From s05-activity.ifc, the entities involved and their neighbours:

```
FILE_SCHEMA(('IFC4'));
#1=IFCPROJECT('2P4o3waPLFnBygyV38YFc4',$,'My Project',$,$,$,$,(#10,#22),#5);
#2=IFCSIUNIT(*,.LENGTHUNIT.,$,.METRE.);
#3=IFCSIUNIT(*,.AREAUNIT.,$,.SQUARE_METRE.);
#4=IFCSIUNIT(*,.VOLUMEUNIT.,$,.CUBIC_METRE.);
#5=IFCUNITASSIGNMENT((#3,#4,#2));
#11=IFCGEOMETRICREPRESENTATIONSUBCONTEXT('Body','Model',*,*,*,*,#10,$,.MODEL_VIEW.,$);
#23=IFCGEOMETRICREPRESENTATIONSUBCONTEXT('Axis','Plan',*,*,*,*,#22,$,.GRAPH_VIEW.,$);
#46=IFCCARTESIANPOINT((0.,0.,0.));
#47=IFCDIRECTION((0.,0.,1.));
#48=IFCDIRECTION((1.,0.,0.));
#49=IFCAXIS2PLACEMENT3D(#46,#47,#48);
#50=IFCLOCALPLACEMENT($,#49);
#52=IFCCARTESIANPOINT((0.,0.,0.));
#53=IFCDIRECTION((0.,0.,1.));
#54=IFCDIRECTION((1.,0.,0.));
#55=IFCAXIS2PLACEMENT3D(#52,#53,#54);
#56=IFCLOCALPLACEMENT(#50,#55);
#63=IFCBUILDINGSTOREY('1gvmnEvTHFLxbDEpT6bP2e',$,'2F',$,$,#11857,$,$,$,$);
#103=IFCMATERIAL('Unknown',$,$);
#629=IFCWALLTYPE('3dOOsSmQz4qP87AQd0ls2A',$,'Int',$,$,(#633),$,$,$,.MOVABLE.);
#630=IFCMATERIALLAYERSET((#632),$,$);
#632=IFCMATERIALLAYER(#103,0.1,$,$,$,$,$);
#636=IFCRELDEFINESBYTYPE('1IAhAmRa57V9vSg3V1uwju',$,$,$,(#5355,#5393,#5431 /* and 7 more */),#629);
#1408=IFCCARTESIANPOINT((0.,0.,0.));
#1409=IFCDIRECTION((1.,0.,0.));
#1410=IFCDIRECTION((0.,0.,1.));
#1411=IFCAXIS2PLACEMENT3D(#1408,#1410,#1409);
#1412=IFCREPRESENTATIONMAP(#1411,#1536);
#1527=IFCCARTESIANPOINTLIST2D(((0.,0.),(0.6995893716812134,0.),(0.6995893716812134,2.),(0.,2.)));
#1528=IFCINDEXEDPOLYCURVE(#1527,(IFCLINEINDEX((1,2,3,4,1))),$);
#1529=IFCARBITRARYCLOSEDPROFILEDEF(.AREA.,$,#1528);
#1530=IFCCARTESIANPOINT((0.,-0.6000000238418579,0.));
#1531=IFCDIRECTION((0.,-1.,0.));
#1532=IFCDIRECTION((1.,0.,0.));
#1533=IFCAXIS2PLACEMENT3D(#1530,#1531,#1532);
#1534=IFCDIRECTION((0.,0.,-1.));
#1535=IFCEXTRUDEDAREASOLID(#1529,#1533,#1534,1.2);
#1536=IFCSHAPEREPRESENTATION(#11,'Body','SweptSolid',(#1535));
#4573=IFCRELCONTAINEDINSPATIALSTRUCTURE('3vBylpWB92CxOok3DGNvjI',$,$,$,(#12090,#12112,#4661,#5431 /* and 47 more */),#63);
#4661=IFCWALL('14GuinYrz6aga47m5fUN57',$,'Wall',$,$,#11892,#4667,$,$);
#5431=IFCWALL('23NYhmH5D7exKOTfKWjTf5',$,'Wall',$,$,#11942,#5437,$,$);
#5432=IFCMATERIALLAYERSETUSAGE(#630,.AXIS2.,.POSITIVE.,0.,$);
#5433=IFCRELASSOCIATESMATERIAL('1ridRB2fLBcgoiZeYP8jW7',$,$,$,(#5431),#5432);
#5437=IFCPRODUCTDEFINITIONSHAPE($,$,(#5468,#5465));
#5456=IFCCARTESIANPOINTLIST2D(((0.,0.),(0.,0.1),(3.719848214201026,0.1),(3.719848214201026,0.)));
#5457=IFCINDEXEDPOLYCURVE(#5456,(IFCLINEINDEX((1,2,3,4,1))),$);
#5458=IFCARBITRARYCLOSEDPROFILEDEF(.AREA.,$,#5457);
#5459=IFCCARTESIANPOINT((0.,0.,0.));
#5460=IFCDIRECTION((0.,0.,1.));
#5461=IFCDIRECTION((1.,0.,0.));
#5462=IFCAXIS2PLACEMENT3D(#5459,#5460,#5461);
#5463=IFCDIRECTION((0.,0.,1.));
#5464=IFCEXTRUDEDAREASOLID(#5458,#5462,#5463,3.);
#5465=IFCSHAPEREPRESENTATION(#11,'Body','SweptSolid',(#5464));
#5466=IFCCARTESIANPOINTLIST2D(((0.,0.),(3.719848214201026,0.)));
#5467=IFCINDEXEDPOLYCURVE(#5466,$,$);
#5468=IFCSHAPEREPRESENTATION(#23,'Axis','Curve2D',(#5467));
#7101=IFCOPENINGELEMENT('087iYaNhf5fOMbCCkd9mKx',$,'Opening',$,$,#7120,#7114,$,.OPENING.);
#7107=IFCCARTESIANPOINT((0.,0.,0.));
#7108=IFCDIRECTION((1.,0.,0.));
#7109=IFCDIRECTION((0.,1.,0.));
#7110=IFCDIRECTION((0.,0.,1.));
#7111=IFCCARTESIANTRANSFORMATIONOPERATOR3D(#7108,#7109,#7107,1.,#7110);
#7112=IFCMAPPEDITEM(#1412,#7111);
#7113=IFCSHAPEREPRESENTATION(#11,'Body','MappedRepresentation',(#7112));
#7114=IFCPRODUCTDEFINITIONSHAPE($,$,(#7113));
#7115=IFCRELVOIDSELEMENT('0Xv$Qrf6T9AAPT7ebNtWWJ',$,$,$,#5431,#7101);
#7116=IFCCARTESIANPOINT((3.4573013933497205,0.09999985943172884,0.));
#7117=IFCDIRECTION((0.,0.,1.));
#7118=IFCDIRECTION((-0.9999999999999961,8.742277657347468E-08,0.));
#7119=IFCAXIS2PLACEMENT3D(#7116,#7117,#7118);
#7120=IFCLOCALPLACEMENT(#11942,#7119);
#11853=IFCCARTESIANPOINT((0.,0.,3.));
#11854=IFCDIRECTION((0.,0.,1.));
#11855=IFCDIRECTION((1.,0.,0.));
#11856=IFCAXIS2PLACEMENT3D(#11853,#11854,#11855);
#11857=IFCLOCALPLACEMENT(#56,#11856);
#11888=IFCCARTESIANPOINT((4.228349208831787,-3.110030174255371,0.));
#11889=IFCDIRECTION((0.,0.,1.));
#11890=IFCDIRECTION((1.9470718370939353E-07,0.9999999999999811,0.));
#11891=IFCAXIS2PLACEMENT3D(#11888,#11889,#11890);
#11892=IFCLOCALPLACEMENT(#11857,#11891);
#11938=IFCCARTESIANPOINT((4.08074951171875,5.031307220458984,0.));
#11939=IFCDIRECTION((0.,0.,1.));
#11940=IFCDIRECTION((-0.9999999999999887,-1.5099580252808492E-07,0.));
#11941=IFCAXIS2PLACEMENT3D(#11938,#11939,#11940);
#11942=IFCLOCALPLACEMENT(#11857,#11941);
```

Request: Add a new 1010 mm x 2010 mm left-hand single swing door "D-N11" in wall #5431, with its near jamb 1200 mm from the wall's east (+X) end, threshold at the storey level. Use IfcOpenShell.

```python
import numpy as np
import ifcopenshell
import ifcopenshell.api.feature
import ifcopenshell.api.geometry
import ifcopenshell.api.root
import ifcopenshell.api.spatial
import ifcopenshell.geom
import ifcopenshell.util.element
import ifcopenshell.util.placement
import ifcopenshell.util.representation
import ifcopenshell.util.shape
import ifcopenshell.util.unit

model = ifcopenshell.open("s05-activity.ifc")
unit_scale = ifcopenshell.util.unit.calculate_unit_scale(model)
settings = ifcopenshell.geom.settings()


def volume(element):
    """Net volume in cubic metres, openings subtracted."""
    shape = ifcopenshell.geom.create_shape(settings, element)
    return ifcopenshell.util.shape.get_volume(shape.geometry)


wall = model.by_guid("23NYhmH5D7exKOTfKWjTf5")
storey = ifcopenshell.util.element.get_container(wall, ifc_class="IfcBuildingStorey")
context = ifcopenshell.util.representation.get_context(model, "Model", "Body", "MODEL_VIEW")
before = volume(wall)

width, height, from_end, sill = 1.01, 2.01, 1.2, 0.0  # metres

# The wall runs along its own X axis, and the end named is its -X end.
wall_shape = ifcopenshell.geom.create_shape(settings, wall)
x, y, z = ifcopenshell.util.shape.get_vertices(wall_shape.geometry).T
start = x.min() + from_end
face, thickness = float(y.min()), float(y.max() - y.min())
wall_matrix = ifcopenshell.util.placement.get_local_placement(wall.ObjectPlacement)
level = ifcopenshell.util.placement.get_local_placement(storey.ObjectPlacement)[2, 3]


def in_wall(x, y):
    """Placement at x, y metres in the wall's axes, at sill height."""
    matrix = wall_matrix.copy()
    matrix[:, 3] = wall_matrix @ np.array([x / unit_scale, y / unit_scale, 0.0, 1.0])
    matrix[2, 3] = level + sill / unit_scale
    return matrix


# Opening: a box that overshoots both wall faces by 50 mm.
opening = ifcopenshell.api.root.create_entity(model, ifc_class="IfcOpeningElement", predefined_type="OPENING")
box = ifcopenshell.api.geometry.add_wall_representation(
    model, context=context, length=width, height=height, thickness=thickness + 0.1
)
ifcopenshell.api.geometry.assign_representation(model, product=opening, representation=box)
ifcopenshell.api.geometry.edit_object_placement(model, product=opening, matrix=in_wall(start, face - 0.05), is_si=False)
ifcopenshell.api.feature.add_feature(model, feature=opening, element=wall)

door = ifcopenshell.api.root.create_entity(model, ifc_class="IfcDoor", name="D-N11", predefined_type="DOOR")
door.OverallWidth, door.OverallHeight = width / unit_scale, height / unit_scale
door.OperationType = "SINGLE_SWING_LEFT"
body = ifcopenshell.api.geometry.add_door_representation(
    model,
    context=context,
    overall_width=door.OverallWidth,
    overall_height=door.OverallHeight,
    operation_type="SINGLE_SWING_LEFT",
    lining_properties={"LiningDepth": thickness / unit_scale, "ThresholdDepth": thickness / unit_scale},
)
ifcopenshell.api.geometry.assign_representation(model, product=door, representation=body)
ifcopenshell.api.spatial.assign_container(model, products=[door], relating_structure=storey)
ifcopenshell.api.feature.add_filling(model, opening=opening, element=door)

# The lining spans the wall, so the door starts at the wall face.
ifcopenshell.api.geometry.edit_object_placement(model, product=door, matrix=in_wall(start, face), is_si=False)

after = volume(wall)

print(f"wall volume {before:.3f} -> {after:.3f} m3")

model.write("s05-activity_updated.ifc")
```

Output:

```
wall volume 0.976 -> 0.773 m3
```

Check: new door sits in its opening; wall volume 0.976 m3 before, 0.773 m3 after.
